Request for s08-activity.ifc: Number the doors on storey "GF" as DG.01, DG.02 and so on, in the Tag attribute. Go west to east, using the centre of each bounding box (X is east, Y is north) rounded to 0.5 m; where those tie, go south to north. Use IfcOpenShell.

First a look at what the model holds.

```python
import ifcopenshell
import ifcopenshell.util.element
import ifcopenshell.util.placement

model = ifcopenshell.open("s08-activity.ifc")
print(model.schema)
storey = next(s for s in model.by_type("IfcBuildingStorey") if s.Name == "GF")
doors = [e for e in ifcopenshell.util.element.get_decomposition(storey) if e.is_a("IfcDoor")]
for e in sorted(doors, key=lambda e: e.id()):
    origin = ifcopenshell.util.placement.get_local_placement(e.ObjectPlacement)[:3, 3]
    print(e.id(), e.Tag, e.Name, origin.round(2) + 0.0, sep=" | ")
```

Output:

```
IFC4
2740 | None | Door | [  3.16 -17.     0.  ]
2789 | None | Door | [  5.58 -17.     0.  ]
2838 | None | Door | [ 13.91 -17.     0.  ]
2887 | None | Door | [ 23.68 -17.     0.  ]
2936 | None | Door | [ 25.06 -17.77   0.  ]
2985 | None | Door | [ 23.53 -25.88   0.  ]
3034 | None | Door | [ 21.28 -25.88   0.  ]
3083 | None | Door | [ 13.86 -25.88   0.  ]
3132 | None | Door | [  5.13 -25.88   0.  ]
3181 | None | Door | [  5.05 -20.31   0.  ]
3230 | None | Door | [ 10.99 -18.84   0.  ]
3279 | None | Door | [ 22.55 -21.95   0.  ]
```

```python
import ifcopenshell
import ifcopenshell.geom
import ifcopenshell.util.element
import ifcopenshell.util.shape

model = ifcopenshell.open("s08-activity.ifc")
settings = ifcopenshell.geom.settings()
settings.set("use-world-coords", True)


def centre(element):
    shape = ifcopenshell.geom.create_shape(settings, element)
    return ifcopenshell.util.shape.get_bbox_centroid(shape.geometry)


storey = next(s for s in model.by_type("IfcBuildingStorey") if s.Name == "GF")
doors = [e for e in ifcopenshell.util.element.get_decomposition(storey) if e.is_a("IfcDoor")]

# Insertion points can sit at a corner or the storey origin, so sort by the geometry (in metres).
centres = {e: centre(e) for e in doors}
doors.sort(key=lambda e: (round(centres[e][0] / 0.5), centres[e][1]))

for i, e in enumerate(doors, start=1):
    number = f"DG.{i:02d}"
    e.Tag = number
    print(e.id(), number)

model.write("s08-activity_edited.ifc")
```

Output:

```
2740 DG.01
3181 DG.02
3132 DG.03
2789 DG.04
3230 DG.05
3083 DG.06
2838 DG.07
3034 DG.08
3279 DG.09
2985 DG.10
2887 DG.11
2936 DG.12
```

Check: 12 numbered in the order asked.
